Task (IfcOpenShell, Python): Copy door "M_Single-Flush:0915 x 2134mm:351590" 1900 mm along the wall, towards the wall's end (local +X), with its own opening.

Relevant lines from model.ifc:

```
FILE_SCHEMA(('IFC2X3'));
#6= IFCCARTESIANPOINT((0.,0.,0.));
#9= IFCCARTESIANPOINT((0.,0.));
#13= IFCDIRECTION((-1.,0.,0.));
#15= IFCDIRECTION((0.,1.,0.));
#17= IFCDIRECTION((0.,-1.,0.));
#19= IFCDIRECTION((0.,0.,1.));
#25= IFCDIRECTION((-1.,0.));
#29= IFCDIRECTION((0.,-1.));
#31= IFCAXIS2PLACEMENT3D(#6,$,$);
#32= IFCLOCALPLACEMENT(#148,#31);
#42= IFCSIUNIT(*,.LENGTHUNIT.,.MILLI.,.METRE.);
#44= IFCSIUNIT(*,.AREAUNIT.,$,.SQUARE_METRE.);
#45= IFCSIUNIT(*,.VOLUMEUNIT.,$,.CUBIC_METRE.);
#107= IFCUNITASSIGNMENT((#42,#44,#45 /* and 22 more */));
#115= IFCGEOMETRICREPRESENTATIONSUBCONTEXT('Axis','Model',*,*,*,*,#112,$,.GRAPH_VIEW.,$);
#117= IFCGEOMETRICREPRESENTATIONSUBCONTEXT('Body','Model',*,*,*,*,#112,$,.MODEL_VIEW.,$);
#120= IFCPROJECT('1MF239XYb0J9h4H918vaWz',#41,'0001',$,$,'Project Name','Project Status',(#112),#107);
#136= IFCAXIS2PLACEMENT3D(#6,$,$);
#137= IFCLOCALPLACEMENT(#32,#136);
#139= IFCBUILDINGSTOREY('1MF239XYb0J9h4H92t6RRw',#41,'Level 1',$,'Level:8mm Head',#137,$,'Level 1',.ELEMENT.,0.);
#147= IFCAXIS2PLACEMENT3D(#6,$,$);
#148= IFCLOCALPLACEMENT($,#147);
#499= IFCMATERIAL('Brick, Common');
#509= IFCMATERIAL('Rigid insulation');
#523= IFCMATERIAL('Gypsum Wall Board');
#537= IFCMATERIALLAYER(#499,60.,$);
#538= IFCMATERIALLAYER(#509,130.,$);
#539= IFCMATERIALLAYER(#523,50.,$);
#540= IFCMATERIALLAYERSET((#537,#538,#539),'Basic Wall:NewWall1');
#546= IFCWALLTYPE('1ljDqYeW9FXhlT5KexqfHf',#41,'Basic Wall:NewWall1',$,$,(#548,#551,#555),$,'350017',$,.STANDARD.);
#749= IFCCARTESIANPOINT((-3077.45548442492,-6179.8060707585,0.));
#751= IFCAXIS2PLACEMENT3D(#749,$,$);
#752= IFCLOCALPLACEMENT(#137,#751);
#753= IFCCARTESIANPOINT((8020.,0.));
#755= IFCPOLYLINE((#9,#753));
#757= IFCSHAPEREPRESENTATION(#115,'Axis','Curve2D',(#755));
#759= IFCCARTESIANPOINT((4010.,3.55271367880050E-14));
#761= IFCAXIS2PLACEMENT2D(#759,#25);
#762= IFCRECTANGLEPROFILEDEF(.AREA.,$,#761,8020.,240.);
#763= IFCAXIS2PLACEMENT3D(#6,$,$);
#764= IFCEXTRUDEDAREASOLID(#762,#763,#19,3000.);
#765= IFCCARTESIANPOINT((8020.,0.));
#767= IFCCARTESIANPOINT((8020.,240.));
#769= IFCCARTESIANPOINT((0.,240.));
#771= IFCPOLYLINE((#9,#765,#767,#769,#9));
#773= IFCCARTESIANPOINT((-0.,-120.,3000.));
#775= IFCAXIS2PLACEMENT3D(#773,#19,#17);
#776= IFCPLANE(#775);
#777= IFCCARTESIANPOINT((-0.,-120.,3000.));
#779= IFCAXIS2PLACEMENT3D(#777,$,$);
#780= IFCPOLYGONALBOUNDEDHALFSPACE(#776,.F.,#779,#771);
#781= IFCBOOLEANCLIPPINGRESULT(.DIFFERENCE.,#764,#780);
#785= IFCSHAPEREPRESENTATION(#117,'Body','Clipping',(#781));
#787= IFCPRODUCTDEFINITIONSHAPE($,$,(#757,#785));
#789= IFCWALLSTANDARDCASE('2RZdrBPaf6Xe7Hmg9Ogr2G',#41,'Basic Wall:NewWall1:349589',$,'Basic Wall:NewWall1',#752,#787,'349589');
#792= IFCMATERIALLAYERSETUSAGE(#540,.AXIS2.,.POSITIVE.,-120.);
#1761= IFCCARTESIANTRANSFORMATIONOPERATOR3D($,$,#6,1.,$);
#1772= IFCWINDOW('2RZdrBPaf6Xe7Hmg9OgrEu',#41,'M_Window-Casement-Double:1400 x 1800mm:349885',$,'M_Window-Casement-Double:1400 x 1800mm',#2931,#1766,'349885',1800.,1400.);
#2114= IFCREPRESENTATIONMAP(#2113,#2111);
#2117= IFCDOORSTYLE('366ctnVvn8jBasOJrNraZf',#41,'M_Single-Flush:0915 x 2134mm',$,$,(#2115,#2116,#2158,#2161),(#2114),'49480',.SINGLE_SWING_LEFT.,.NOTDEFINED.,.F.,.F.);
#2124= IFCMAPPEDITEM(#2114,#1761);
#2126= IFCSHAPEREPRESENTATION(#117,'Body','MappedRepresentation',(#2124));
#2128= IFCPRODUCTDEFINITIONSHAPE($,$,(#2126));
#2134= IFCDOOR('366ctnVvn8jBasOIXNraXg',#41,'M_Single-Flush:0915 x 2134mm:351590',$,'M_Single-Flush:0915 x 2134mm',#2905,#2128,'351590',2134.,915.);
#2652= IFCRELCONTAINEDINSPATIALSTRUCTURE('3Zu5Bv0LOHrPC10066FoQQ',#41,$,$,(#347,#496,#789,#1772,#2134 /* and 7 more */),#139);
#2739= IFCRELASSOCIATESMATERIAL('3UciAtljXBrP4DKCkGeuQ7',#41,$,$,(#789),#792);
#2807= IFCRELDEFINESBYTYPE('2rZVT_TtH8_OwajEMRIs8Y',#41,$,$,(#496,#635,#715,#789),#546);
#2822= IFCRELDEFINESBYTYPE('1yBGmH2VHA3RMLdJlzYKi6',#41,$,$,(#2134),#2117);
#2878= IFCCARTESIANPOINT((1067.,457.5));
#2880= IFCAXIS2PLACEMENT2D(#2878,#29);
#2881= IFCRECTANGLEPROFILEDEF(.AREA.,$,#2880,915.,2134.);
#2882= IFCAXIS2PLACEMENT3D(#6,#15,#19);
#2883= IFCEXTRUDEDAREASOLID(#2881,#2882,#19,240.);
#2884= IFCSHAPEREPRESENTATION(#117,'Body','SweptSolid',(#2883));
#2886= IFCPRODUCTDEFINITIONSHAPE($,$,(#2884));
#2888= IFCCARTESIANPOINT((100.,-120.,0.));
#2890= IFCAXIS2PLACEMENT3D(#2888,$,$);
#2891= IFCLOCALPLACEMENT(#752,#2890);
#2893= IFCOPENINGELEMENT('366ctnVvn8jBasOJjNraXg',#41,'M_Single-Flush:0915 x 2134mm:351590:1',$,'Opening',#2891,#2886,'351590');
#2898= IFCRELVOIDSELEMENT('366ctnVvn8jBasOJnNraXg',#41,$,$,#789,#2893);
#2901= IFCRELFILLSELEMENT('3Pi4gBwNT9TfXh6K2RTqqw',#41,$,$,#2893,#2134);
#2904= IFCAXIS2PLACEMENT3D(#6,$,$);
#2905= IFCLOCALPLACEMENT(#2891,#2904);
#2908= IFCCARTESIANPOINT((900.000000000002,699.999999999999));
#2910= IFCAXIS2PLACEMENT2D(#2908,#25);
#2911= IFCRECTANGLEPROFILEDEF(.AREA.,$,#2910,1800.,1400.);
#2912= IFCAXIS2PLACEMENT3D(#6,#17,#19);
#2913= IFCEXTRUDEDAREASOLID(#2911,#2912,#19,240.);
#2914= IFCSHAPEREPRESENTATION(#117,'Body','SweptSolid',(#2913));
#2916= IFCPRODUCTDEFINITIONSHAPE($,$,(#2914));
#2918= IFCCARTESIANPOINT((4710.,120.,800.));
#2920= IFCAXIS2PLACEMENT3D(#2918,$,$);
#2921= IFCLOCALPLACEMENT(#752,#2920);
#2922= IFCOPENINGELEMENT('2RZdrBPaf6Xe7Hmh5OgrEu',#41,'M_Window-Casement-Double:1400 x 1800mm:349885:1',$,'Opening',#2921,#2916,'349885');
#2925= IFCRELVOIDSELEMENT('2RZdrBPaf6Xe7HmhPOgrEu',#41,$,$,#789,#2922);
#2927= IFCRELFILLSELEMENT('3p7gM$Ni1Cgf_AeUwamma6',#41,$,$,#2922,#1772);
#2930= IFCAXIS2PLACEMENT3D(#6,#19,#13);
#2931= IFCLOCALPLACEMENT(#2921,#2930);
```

```python
import ifcopenshell
import ifcopenshell.api.feature
import ifcopenshell.api.geometry
import ifcopenshell.api.root
import ifcopenshell.geom
import ifcopenshell.util.element
import ifcopenshell.util.placement
import ifcopenshell.util.shape

model = ifcopenshell.open("model.ifc")
settings = ifcopenshell.geom.settings()


def volume(element):
    """Net volume in cubic metres, openings subtracted."""
    shape = ifcopenshell.geom.create_shape(settings, element)
    return ifcopenshell.util.shape.get_volume(shape.geometry)


def reuse_history(source, copy):
    """copy_class also copies each property set's owner history, people and application; keep the originals."""
    for rel in copy.IsDefinedBy:
        if rel.is_a("IfcRelDefinesByProperties") and (history := rel.RelatingPropertyDefinition.OwnerHistory):
            rel.RelatingPropertyDefinition.OwnerHistory = source.OwnerHistory
            ifcopenshell.util.element.remove_deep2(model, history)


door = model.by_guid("366ctnVvn8jBasOIXNraXg")
opening = door.FillsVoids[0].RelatingOpeningElement
wall = opening.VoidsElements[0].RelatingBuildingElement
before = volume(wall)
shift = ifcopenshell.util.placement.get_local_placement(wall.ObjectPlacement)[:3, 0] * 1900.0

# copy_class copies the void relationship, type, container and properties, but no geometry.
new_opening = ifcopenshell.api.root.copy_class(model, product=opening)
new_opening.Representation = ifcopenshell.util.element.copy_deep(
    model, opening.Representation, exclude=["IfcGeometricRepresentationContext", "IfcRepresentationMap"]
)
new_opening.Name = "M_Single-Flush:0915 x 2134mm"
new_opening.Tag = None
new_door = ifcopenshell.api.root.copy_class(model, product=door)
new_door.Representation = ifcopenshell.util.element.copy_deep(
    model, door.Representation, exclude=["IfcGeometricRepresentationContext", "IfcRepresentationMap"]
)
new_door.Name = "M_Single-Flush:0915 x 2134mm"
new_door.Tag = None
reuse_history(door, new_door)
fills = ifcopenshell.api.feature.add_filling(model, opening=new_opening, element=new_door)
fills.OwnerHistory = new_door.OwnerHistory  # required in IFC2X3

for old, new in ((opening, new_opening), (door, new_door)):
    matrix = ifcopenshell.util.placement.get_local_placement(old.ObjectPlacement)
    matrix[:3, 3] += shift
    ifcopenshell.api.geometry.edit_object_placement(model, product=new, matrix=matrix, is_si=False)

after = volume(wall)

print(f"wall volume {before:.3f} -> {after:.3f} m3")

model.write("model-out.ifc")
```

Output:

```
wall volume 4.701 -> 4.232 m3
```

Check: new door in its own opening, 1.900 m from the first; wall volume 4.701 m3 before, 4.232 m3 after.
